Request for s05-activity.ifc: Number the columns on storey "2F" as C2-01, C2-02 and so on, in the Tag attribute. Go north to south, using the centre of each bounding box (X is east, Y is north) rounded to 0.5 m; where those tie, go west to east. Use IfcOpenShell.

First a look at what the model holds.

```python
import ifcopenshell
import ifcopenshell.util.element
import ifcopenshell.util.placement

model = ifcopenshell.open("s05-activity.ifc")
print(model.schema)
storey = next(s for s in model.by_type("IfcBuildingStorey") if s.Name == "2F")
columns = [e for e in ifcopenshell.util.element.get_decomposition(storey) if e.is_a("IfcColumn")]
for e in sorted(columns, key=lambda e: e.id()):
    origin = ifcopenshell.util.placement.get_local_placement(e.ObjectPlacement)[:3, 3]
    print(e.id(), e.Tag, e.Name, origin.round(2) + 0.0, sep=" | ")
```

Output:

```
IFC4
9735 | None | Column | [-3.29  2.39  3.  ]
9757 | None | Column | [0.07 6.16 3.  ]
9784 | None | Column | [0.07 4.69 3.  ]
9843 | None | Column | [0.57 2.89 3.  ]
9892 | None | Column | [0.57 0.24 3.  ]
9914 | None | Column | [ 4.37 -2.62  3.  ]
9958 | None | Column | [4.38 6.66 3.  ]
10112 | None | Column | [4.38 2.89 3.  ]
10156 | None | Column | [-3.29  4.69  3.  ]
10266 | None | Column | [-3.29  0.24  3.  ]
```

```python
import ifcopenshell
import ifcopenshell.geom
import ifcopenshell.util.element
import ifcopenshell.util.shape

model = ifcopenshell.open("s05-activity.ifc")
settings = ifcopenshell.geom.settings()
settings.set("use-world-coords", True)


def centre(element):
    shape = ifcopenshell.geom.create_shape(settings, element)
    return ifcopenshell.util.shape.get_bbox_centroid(shape.geometry)


storey = next(s for s in model.by_type("IfcBuildingStorey") if s.Name == "2F")
columns = [e for e in ifcopenshell.util.element.get_decomposition(storey) if e.is_a("IfcColumn")]

# Insertion points can sit at a corner or the storey origin, so sort by the geometry (in metres).
centres = {e: centre(e) for e in columns}
columns.sort(key=lambda e: (-round(centres[e][1] / 0.5), centres[e][0]))

for i, e in enumerate(columns, start=1):
    number = f"C2-{i:02d}"
    e.Tag = number
    print(e.id(), number)

model.write("s05-activity_edited.ifc")
```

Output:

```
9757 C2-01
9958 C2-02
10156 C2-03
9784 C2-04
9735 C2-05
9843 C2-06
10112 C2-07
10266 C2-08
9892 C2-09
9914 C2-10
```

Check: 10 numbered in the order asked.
